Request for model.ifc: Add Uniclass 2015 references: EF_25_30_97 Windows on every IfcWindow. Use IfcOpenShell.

First a look at what the model holds.

```python
import ifcopenshell

model = ifcopenshell.open("model.ifc")
print(model.schema)
print("classifications:", [c.Name for c in model.by_type("IfcClassification")])
for ifc_class in ("IfcDoor", "IfcRoof", "IfcStair", "IfcWall", "IfcWindow"):
    print(ifc_class, len(model.by_type(ifc_class)))
```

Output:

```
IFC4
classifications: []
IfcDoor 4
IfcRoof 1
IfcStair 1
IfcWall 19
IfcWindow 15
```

```python
import ifcopenshell
import ifcopenshell.api.classification

model = ifcopenshell.open("model.ifc")

system = ifcopenshell.api.classification.add_classification(model, classification="Uniclass 2015")

codes = {
    "IfcWindow": ("EF_25_30_97", "Windows"),
}
for ifc_class, (code, name) in codes.items():
    products = model.by_type(ifc_class)
    ifcopenshell.api.classification.add_reference(
        model, products=products, classification=system, identification=code, name=name
    )
    print(code, len(products))

model.write("model_rev.ifc")
```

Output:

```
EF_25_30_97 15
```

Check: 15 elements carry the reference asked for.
